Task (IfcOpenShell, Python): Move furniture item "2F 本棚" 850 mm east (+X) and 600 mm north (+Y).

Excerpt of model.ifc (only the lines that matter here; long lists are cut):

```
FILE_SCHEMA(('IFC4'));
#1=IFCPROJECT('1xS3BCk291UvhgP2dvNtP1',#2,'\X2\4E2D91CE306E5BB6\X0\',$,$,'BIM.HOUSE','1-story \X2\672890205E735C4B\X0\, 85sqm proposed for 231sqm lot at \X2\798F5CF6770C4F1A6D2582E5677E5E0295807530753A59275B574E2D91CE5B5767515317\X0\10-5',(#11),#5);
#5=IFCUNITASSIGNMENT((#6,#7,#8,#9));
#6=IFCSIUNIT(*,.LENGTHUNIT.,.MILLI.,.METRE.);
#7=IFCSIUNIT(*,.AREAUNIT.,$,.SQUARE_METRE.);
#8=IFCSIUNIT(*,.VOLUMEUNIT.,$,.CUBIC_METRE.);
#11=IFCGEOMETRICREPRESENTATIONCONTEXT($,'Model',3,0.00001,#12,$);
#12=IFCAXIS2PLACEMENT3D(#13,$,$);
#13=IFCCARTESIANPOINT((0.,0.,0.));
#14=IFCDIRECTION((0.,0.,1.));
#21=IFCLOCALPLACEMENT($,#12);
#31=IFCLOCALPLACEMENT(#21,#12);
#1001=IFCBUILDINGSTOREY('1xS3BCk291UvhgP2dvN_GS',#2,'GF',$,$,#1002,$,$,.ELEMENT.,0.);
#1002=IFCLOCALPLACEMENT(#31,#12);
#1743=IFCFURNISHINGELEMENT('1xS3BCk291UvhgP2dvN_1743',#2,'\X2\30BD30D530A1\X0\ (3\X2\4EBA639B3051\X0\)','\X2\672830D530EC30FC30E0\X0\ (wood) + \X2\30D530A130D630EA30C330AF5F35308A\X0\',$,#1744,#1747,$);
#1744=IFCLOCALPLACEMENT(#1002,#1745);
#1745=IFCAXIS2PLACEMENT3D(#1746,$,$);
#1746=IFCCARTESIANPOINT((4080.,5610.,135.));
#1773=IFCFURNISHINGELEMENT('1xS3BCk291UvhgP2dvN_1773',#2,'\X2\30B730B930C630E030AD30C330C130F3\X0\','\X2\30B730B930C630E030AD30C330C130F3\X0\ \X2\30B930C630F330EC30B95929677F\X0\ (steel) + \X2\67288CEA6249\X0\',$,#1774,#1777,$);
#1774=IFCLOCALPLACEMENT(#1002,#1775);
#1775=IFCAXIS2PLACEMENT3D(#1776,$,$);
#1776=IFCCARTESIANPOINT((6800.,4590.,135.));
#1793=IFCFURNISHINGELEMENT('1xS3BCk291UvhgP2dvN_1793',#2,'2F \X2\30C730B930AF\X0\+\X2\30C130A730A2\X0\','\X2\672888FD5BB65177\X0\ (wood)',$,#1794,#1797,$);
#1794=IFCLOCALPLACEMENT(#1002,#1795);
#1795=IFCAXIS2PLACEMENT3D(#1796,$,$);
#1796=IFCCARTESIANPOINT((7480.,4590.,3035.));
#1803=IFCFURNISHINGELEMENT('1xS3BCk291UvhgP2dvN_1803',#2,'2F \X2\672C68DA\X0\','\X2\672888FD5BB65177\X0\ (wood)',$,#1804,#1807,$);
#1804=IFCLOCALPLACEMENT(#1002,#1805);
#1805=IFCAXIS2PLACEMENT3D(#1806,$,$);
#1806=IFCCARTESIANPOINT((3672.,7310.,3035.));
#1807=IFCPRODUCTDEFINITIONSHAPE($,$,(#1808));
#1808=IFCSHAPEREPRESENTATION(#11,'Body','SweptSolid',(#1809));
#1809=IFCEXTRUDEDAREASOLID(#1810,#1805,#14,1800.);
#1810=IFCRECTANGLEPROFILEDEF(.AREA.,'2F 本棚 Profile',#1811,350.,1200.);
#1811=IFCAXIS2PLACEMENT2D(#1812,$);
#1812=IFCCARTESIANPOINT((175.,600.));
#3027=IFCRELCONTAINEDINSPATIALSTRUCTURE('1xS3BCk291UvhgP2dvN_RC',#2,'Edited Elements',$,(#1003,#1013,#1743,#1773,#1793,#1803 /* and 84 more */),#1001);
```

```python
import ifcopenshell
import ifcopenshell.api.geometry
import ifcopenshell.util.placement

model = ifcopenshell.open("model.ifc")

item = model.by_guid("1xS3BCk291UvhgP2dvN_1803")
matrix = ifcopenshell.util.placement.get_local_placement(item.ObjectPlacement)
matrix[0, 3] += 850.0
matrix[1, 3] += 600.0
ifcopenshell.api.geometry.edit_object_placement(model, product=item, matrix=matrix, is_si=False)

print(ifcopenshell.util.placement.get_local_placement(item.ObjectPlacement).round(3) + 0.0)

model.write("model-out.ifc")
```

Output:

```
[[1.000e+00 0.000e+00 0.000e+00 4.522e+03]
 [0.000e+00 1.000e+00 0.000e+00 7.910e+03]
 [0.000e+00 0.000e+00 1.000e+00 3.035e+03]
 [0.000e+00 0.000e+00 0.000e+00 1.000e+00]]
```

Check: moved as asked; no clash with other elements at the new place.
